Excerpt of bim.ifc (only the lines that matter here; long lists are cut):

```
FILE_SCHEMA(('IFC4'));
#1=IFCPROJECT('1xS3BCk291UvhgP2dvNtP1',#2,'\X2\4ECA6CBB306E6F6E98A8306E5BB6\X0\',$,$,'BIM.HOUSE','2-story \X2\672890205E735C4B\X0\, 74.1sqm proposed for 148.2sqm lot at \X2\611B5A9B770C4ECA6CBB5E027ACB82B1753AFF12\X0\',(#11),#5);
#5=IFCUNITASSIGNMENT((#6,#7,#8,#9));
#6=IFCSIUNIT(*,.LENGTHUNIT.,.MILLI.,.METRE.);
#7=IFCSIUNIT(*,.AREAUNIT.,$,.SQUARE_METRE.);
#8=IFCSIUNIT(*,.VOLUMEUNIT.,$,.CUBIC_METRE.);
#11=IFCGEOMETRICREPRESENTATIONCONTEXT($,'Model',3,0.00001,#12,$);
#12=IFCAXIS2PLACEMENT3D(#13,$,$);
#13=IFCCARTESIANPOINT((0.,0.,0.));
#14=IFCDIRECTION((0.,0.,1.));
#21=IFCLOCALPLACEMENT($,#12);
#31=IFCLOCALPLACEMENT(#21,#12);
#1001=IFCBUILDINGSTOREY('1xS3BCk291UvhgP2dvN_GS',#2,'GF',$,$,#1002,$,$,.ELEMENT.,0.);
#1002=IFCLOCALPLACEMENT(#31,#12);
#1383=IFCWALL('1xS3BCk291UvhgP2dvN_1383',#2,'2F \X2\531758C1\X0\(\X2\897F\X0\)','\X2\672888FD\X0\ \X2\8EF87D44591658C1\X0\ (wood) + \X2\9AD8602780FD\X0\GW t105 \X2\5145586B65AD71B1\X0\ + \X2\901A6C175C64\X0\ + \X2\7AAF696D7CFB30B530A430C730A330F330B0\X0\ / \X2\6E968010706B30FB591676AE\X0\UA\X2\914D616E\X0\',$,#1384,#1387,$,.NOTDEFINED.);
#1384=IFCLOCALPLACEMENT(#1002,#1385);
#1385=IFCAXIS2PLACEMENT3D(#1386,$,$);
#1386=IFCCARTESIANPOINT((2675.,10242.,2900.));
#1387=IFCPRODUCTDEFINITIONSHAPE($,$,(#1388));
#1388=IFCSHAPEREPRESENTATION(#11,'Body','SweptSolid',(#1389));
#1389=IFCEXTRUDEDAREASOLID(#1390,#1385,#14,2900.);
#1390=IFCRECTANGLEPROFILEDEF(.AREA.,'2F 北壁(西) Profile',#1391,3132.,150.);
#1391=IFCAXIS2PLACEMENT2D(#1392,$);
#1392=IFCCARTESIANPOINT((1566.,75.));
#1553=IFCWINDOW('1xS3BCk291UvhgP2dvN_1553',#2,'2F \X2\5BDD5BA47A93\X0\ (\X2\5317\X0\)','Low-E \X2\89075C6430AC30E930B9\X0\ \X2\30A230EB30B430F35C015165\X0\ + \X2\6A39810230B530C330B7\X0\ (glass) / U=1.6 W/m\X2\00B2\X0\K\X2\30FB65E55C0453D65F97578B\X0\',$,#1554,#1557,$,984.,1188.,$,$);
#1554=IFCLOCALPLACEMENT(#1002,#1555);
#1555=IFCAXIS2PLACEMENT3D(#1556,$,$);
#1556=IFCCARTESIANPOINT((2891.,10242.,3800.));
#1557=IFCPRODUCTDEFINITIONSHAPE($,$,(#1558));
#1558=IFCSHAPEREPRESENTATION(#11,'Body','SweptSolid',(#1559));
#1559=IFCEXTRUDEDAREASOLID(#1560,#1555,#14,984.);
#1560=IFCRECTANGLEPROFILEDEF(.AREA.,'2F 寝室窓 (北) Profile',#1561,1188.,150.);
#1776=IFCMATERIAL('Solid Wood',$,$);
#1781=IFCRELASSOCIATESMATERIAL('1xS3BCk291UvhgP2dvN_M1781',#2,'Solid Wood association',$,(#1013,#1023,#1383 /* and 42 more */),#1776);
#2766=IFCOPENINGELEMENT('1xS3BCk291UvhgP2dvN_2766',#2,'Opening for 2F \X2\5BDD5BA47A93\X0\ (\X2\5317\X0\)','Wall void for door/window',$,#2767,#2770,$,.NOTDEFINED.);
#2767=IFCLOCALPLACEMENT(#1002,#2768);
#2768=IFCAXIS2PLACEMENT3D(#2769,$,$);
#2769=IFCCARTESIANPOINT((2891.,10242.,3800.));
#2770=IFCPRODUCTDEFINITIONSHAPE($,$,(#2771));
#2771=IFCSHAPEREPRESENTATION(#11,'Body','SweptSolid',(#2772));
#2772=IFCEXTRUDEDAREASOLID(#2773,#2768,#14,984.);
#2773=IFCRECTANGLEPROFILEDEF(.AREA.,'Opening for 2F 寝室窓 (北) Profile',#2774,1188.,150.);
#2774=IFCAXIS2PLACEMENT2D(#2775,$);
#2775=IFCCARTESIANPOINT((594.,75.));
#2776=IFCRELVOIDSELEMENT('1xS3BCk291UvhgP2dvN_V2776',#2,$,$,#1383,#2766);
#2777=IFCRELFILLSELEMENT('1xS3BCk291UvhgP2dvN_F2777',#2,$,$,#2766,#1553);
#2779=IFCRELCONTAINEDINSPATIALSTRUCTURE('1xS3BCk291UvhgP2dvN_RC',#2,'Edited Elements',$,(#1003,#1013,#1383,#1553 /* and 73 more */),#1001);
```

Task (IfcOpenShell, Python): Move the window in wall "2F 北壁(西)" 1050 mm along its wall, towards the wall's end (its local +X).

```python
import ifcopenshell
import ifcopenshell.api.geometry
import ifcopenshell.util.placement
import ifcopenshell.util.unit

model = ifcopenshell.open("bim.ifc")
unit_scale = ifcopenshell.util.unit.calculate_unit_scale(model)

window = model.by_guid("1xS3BCk291UvhgP2dvN_1553")
opening = window.FillsVoids[0].RelatingOpeningElement
wall = opening.VoidsElements[0].RelatingBuildingElement

wall_matrix = ifcopenshell.util.placement.get_local_placement(wall.ObjectPlacement)
shift = wall_matrix[:3, 0] * 1.05 / unit_scale
before = ifcopenshell.util.placement.get_local_placement(window.ObjectPlacement)[:3, 3].copy()

# The window is not placed relative to its opening, so move both.
for product in (opening, window):
    matrix = ifcopenshell.util.placement.get_local_placement(product.ObjectPlacement)
    matrix[:3, 3] += shift
    ifcopenshell.api.geometry.edit_object_placement(model, product=product, matrix=matrix, is_si=False)

after = ifcopenshell.util.placement.get_local_placement(window.ObjectPlacement)[:3, 3]
print("window moved by", (after - before).round(3) + 0.0)

model.write("bim_rev.ifc")
```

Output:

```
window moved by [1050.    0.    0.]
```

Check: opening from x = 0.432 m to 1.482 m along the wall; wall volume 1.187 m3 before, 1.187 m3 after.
